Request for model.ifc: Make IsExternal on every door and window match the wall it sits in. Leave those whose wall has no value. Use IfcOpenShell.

First a look at what the model holds.

```python
import ifcopenshell
import ifcopenshell.util.element

model = ifcopenshell.open("model.ifc")
print(model.schema)
seen = {}
for e in model.by_type("IfcDoor") + model.by_type("IfcWindow"):
    if not e.FillsVoids:
        continue
    host = e.FillsVoids[0].RelatingOpeningElement.VoidsElements[0].RelatingBuildingElement
    own = ifcopenshell.util.element.get_pset(e, f"Pset_{e.is_a()[3:].removesuffix('StandardCase')}Common", "IsExternal")
    wall = ifcopenshell.util.element.get_pset(host, "Pset_WallCommon", "IsExternal")
    seen[e.is_a(), own, wall] = seen.get((e.is_a(), own, wall), 0) + 1
for (cls, own, wall), count in sorted(seen.items(), key=str):
    print(count, cls, "IsExternal:", own, "| host wall:", wall)
```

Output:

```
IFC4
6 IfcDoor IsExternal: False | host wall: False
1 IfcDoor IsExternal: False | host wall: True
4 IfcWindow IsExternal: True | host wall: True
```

```python
import ifcopenshell
import ifcopenshell.api.pset
import ifcopenshell.util.element

model = ifcopenshell.open("model.ifc")

count = 0
for ifc_class, pset_name in (("IfcDoor", "Pset_DoorCommon"), ("IfcWindow", "Pset_WindowCommon")):
    for e in model.by_type(ifc_class):
        if not e.FillsVoids:
            continue
        host = e.FillsVoids[0].RelatingOpeningElement.VoidsElements[0].RelatingBuildingElement
        external = ifcopenshell.util.element.get_pset(host, "Pset_WallCommon", "IsExternal")
        if external is None or ifcopenshell.util.element.get_pset(e, pset_name, "IsExternal") == external:
            continue
        pset = ifcopenshell.api.pset.add_pset(model, product=e, name=pset_name)
        ifcopenshell.api.pset.edit_pset(model, pset=pset, properties={"IsExternal": external})
        count += 1

print(count, "updated")

model.write("model_rev.ifc")
```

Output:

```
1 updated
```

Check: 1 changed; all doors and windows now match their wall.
